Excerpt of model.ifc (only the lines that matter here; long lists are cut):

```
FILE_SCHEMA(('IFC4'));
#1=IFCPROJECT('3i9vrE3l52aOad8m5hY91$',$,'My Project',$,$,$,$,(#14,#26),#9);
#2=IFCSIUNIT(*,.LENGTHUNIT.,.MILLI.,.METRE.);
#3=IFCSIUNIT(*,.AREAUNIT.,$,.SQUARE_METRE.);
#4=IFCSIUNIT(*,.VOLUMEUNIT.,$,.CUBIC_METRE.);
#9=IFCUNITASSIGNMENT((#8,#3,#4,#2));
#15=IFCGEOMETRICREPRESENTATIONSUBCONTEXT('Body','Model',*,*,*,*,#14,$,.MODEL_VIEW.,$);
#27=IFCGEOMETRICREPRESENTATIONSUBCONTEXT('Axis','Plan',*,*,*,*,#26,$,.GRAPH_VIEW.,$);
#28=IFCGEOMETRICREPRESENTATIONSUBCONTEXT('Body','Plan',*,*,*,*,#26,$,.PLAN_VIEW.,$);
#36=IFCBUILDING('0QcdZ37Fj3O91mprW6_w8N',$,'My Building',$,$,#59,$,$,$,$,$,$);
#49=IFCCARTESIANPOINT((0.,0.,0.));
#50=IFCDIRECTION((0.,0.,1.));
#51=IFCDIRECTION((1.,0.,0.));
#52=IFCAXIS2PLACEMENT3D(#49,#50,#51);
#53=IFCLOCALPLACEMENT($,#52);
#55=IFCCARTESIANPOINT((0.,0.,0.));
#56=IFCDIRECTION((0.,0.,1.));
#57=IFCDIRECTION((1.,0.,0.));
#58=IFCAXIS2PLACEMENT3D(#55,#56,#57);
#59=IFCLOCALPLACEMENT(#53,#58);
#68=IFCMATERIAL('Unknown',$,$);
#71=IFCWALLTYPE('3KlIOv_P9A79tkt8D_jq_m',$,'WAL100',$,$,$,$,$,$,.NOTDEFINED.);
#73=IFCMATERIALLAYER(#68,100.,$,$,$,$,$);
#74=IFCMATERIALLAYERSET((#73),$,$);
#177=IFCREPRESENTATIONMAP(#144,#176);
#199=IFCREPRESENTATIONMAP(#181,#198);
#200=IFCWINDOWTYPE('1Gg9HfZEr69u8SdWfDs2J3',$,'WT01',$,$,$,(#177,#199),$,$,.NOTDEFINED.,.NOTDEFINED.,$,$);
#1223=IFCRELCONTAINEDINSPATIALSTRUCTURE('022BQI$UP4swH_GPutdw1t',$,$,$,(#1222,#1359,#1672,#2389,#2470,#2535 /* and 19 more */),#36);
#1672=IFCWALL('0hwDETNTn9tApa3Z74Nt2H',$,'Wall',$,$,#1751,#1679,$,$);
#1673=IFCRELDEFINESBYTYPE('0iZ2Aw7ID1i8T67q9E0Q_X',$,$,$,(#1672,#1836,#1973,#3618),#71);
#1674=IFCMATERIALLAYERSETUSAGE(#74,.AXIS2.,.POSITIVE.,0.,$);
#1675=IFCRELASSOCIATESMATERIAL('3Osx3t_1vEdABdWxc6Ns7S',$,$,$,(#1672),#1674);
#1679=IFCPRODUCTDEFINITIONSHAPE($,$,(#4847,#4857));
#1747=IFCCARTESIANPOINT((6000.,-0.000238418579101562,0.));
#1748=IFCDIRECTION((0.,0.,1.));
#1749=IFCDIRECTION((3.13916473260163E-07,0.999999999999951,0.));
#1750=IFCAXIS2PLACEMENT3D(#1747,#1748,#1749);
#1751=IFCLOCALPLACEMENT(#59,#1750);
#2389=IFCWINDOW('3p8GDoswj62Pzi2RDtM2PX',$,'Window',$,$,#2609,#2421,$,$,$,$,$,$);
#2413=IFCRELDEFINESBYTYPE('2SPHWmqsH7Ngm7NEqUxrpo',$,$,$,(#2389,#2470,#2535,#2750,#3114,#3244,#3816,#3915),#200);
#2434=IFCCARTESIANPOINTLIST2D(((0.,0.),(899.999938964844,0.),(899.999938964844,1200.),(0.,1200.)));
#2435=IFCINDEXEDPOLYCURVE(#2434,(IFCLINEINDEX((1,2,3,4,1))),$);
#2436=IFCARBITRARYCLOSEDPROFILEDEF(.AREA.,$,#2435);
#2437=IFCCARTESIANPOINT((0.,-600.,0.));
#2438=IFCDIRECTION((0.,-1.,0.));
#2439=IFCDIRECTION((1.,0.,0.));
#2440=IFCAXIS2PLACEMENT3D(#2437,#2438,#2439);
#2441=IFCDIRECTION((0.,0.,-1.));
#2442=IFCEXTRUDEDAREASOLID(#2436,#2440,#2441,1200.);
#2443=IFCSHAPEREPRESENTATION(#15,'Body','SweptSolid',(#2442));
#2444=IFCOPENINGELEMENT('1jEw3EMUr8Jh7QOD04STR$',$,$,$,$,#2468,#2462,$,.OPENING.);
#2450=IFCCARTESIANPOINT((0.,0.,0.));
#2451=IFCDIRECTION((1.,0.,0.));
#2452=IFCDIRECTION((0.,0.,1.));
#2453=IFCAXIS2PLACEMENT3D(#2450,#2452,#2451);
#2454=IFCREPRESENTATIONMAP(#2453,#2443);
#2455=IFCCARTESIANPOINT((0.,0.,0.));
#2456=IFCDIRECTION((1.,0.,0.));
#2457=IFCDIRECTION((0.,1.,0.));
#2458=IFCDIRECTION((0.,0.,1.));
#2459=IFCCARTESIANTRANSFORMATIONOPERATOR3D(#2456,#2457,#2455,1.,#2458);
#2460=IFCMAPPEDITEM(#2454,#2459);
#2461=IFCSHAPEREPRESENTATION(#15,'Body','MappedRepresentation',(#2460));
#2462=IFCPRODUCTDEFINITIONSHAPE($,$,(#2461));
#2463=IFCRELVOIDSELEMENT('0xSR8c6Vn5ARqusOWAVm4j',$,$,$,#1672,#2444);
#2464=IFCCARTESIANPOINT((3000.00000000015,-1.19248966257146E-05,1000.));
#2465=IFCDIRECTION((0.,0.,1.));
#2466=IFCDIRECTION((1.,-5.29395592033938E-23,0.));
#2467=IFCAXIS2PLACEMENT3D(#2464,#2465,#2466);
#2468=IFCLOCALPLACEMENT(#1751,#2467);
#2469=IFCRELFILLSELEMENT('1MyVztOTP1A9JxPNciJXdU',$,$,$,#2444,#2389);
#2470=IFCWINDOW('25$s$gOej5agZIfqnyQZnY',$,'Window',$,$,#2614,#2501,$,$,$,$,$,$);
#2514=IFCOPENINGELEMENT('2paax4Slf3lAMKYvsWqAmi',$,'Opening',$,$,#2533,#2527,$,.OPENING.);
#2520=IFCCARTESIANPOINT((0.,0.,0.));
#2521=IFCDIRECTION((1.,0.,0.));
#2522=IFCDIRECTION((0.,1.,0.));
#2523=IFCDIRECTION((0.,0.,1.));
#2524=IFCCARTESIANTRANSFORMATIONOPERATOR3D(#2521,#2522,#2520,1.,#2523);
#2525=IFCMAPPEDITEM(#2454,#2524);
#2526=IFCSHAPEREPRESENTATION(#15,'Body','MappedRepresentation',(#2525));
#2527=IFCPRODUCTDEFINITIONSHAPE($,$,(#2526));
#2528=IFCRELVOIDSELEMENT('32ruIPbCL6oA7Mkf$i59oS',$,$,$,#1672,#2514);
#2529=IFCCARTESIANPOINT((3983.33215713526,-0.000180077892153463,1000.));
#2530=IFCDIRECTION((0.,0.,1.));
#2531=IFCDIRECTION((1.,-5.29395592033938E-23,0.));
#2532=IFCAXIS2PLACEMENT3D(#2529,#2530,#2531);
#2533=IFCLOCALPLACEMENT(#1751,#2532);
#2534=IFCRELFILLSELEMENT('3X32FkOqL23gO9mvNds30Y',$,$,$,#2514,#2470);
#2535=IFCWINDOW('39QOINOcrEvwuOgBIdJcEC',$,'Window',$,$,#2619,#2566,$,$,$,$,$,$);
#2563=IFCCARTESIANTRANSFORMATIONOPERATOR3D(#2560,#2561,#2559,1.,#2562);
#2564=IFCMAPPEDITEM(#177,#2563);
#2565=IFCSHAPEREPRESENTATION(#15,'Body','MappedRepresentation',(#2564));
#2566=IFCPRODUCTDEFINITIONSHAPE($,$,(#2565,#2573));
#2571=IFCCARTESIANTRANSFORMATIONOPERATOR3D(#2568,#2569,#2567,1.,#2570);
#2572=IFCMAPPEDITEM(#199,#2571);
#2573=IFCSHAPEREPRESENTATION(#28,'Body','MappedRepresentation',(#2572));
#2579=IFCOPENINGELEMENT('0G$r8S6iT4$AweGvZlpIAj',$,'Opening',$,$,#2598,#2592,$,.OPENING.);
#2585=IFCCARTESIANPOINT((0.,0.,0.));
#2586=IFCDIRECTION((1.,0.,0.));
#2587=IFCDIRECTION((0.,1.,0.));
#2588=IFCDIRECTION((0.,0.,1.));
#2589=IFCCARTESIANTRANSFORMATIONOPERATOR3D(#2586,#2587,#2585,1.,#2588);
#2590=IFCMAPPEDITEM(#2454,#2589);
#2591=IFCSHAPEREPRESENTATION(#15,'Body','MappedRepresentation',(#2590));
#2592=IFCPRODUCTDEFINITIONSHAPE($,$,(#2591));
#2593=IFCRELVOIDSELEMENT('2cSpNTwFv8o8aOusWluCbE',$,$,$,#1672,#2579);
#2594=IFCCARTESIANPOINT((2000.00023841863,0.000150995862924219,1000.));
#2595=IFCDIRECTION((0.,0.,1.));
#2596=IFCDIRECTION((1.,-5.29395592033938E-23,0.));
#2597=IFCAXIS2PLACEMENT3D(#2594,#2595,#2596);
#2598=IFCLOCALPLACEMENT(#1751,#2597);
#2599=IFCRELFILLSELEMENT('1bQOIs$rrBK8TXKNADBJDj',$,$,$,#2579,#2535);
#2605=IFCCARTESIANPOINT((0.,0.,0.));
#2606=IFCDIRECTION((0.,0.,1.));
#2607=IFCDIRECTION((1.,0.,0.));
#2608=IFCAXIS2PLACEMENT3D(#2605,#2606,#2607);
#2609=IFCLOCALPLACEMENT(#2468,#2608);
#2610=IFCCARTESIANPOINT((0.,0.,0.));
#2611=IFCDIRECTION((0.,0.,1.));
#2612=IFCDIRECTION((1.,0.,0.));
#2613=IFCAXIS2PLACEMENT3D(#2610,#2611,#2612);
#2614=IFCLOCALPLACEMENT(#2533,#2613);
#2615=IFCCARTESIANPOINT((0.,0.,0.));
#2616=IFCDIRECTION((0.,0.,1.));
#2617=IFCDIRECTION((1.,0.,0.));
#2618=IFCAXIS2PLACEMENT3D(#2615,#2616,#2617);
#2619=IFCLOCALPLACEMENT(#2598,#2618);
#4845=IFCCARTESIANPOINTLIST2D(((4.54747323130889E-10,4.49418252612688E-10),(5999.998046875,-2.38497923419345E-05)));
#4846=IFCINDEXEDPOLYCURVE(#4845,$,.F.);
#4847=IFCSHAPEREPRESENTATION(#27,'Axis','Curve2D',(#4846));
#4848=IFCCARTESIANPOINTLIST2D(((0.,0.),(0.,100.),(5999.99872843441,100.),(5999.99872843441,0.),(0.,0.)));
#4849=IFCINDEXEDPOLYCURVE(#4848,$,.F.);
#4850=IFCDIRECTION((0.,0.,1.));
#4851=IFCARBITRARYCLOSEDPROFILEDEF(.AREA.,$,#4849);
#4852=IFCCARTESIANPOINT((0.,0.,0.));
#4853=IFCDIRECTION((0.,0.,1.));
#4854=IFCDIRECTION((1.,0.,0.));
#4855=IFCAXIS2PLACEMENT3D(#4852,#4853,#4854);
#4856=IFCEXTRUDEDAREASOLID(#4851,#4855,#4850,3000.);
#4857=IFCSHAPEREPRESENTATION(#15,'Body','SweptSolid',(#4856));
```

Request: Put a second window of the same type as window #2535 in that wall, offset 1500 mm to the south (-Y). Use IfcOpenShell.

```python
import ifcopenshell
import ifcopenshell.api.feature
import ifcopenshell.api.geometry
import ifcopenshell.api.root
import ifcopenshell.geom
import ifcopenshell.util.element
import ifcopenshell.util.placement
import ifcopenshell.util.shape

model = ifcopenshell.open("model.ifc")
settings = ifcopenshell.geom.settings()


def volume(element):
    """Net volume in cubic metres, openings subtracted."""
    shape = ifcopenshell.geom.create_shape(settings, element)
    return ifcopenshell.util.shape.get_volume(shape.geometry)


window = model.by_guid("39QOINOcrEvwuOgBIdJcEC")
opening = window.FillsVoids[0].RelatingOpeningElement
wall = opening.VoidsElements[0].RelatingBuildingElement
before = volume(wall)
shift = ifcopenshell.util.placement.get_local_placement(wall.ObjectPlacement)[:3, 0] * -1500.0

# copy_class copies the void relationship, type, container and properties, but no geometry.
new_opening = ifcopenshell.api.root.copy_class(model, product=opening)
new_opening.Representation = ifcopenshell.util.element.copy_deep(
    model, opening.Representation, exclude=["IfcGeometricRepresentationContext", "IfcRepresentationMap"]
)
new_window = ifcopenshell.api.root.copy_class(model, product=window)
new_window.Representation = ifcopenshell.util.element.copy_deep(
    model, window.Representation, exclude=["IfcGeometricRepresentationContext", "IfcRepresentationMap"]
)
ifcopenshell.api.feature.add_filling(model, opening=new_opening, element=new_window)

for old, new in ((opening, new_opening), (window, new_window)):
    matrix = ifcopenshell.util.placement.get_local_placement(old.ObjectPlacement)
    matrix[:3, 3] += shift
    ifcopenshell.api.geometry.edit_object_placement(model, product=new, matrix=matrix, is_si=False)

after = volume(wall)

print(f"wall volume {before:.3f} -> {after:.3f} m3")

model.write("model_rev.ifc")
```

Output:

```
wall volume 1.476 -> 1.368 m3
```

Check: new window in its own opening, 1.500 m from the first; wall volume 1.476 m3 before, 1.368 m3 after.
